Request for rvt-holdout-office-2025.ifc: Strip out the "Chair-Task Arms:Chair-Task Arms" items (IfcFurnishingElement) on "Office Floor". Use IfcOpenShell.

First a look at what the model holds.

```python
import ifcopenshell
import ifcopenshell.util.element

model = ifcopenshell.open("rvt-holdout-office-2025.ifc")
print(model.schema)
storey = next(s for s in model.by_type("IfcBuildingStorey") if s.Name == "Office Floor")
furniture = [e for e in ifcopenshell.util.element.get_decomposition(storey) if e.is_a("IfcFurnishingElement")]
seen = {}
for e in furniture:
    element_type = ifcopenshell.util.element.get_type(e)
    name = element_type.Name if element_type not in (None, e) else None
    seen[name] = seen.get(name, 0) + 1
for name, count in sorted(seen.items(), key=str):
    print(count, "x", name)
```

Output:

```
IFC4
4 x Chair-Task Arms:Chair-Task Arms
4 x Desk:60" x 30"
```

```python
import ifcopenshell
import ifcopenshell.api.root
import ifcopenshell.util.element

model = ifcopenshell.open("rvt-holdout-office-2025.ifc")

storey = next(s for s in model.by_type("IfcBuildingStorey") if s.Name == "Office Floor")
furniture = [e for e in ifcopenshell.util.element.get_decomposition(storey) if e.is_a("IfcFurnishingElement")]
targets = [e for e in furniture if (t := ifcopenshell.util.element.get_type(e)) not in (None, e) and t.Name == "Chair-Task Arms:Chair-Task Arms"]

for e in targets:
    ifcopenshell.api.root.remove_product(model, product=e)
print(len(targets), "removed")

model.write("rvt-holdout-office-2025_edited.ifc")
```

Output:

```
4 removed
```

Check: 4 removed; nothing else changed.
